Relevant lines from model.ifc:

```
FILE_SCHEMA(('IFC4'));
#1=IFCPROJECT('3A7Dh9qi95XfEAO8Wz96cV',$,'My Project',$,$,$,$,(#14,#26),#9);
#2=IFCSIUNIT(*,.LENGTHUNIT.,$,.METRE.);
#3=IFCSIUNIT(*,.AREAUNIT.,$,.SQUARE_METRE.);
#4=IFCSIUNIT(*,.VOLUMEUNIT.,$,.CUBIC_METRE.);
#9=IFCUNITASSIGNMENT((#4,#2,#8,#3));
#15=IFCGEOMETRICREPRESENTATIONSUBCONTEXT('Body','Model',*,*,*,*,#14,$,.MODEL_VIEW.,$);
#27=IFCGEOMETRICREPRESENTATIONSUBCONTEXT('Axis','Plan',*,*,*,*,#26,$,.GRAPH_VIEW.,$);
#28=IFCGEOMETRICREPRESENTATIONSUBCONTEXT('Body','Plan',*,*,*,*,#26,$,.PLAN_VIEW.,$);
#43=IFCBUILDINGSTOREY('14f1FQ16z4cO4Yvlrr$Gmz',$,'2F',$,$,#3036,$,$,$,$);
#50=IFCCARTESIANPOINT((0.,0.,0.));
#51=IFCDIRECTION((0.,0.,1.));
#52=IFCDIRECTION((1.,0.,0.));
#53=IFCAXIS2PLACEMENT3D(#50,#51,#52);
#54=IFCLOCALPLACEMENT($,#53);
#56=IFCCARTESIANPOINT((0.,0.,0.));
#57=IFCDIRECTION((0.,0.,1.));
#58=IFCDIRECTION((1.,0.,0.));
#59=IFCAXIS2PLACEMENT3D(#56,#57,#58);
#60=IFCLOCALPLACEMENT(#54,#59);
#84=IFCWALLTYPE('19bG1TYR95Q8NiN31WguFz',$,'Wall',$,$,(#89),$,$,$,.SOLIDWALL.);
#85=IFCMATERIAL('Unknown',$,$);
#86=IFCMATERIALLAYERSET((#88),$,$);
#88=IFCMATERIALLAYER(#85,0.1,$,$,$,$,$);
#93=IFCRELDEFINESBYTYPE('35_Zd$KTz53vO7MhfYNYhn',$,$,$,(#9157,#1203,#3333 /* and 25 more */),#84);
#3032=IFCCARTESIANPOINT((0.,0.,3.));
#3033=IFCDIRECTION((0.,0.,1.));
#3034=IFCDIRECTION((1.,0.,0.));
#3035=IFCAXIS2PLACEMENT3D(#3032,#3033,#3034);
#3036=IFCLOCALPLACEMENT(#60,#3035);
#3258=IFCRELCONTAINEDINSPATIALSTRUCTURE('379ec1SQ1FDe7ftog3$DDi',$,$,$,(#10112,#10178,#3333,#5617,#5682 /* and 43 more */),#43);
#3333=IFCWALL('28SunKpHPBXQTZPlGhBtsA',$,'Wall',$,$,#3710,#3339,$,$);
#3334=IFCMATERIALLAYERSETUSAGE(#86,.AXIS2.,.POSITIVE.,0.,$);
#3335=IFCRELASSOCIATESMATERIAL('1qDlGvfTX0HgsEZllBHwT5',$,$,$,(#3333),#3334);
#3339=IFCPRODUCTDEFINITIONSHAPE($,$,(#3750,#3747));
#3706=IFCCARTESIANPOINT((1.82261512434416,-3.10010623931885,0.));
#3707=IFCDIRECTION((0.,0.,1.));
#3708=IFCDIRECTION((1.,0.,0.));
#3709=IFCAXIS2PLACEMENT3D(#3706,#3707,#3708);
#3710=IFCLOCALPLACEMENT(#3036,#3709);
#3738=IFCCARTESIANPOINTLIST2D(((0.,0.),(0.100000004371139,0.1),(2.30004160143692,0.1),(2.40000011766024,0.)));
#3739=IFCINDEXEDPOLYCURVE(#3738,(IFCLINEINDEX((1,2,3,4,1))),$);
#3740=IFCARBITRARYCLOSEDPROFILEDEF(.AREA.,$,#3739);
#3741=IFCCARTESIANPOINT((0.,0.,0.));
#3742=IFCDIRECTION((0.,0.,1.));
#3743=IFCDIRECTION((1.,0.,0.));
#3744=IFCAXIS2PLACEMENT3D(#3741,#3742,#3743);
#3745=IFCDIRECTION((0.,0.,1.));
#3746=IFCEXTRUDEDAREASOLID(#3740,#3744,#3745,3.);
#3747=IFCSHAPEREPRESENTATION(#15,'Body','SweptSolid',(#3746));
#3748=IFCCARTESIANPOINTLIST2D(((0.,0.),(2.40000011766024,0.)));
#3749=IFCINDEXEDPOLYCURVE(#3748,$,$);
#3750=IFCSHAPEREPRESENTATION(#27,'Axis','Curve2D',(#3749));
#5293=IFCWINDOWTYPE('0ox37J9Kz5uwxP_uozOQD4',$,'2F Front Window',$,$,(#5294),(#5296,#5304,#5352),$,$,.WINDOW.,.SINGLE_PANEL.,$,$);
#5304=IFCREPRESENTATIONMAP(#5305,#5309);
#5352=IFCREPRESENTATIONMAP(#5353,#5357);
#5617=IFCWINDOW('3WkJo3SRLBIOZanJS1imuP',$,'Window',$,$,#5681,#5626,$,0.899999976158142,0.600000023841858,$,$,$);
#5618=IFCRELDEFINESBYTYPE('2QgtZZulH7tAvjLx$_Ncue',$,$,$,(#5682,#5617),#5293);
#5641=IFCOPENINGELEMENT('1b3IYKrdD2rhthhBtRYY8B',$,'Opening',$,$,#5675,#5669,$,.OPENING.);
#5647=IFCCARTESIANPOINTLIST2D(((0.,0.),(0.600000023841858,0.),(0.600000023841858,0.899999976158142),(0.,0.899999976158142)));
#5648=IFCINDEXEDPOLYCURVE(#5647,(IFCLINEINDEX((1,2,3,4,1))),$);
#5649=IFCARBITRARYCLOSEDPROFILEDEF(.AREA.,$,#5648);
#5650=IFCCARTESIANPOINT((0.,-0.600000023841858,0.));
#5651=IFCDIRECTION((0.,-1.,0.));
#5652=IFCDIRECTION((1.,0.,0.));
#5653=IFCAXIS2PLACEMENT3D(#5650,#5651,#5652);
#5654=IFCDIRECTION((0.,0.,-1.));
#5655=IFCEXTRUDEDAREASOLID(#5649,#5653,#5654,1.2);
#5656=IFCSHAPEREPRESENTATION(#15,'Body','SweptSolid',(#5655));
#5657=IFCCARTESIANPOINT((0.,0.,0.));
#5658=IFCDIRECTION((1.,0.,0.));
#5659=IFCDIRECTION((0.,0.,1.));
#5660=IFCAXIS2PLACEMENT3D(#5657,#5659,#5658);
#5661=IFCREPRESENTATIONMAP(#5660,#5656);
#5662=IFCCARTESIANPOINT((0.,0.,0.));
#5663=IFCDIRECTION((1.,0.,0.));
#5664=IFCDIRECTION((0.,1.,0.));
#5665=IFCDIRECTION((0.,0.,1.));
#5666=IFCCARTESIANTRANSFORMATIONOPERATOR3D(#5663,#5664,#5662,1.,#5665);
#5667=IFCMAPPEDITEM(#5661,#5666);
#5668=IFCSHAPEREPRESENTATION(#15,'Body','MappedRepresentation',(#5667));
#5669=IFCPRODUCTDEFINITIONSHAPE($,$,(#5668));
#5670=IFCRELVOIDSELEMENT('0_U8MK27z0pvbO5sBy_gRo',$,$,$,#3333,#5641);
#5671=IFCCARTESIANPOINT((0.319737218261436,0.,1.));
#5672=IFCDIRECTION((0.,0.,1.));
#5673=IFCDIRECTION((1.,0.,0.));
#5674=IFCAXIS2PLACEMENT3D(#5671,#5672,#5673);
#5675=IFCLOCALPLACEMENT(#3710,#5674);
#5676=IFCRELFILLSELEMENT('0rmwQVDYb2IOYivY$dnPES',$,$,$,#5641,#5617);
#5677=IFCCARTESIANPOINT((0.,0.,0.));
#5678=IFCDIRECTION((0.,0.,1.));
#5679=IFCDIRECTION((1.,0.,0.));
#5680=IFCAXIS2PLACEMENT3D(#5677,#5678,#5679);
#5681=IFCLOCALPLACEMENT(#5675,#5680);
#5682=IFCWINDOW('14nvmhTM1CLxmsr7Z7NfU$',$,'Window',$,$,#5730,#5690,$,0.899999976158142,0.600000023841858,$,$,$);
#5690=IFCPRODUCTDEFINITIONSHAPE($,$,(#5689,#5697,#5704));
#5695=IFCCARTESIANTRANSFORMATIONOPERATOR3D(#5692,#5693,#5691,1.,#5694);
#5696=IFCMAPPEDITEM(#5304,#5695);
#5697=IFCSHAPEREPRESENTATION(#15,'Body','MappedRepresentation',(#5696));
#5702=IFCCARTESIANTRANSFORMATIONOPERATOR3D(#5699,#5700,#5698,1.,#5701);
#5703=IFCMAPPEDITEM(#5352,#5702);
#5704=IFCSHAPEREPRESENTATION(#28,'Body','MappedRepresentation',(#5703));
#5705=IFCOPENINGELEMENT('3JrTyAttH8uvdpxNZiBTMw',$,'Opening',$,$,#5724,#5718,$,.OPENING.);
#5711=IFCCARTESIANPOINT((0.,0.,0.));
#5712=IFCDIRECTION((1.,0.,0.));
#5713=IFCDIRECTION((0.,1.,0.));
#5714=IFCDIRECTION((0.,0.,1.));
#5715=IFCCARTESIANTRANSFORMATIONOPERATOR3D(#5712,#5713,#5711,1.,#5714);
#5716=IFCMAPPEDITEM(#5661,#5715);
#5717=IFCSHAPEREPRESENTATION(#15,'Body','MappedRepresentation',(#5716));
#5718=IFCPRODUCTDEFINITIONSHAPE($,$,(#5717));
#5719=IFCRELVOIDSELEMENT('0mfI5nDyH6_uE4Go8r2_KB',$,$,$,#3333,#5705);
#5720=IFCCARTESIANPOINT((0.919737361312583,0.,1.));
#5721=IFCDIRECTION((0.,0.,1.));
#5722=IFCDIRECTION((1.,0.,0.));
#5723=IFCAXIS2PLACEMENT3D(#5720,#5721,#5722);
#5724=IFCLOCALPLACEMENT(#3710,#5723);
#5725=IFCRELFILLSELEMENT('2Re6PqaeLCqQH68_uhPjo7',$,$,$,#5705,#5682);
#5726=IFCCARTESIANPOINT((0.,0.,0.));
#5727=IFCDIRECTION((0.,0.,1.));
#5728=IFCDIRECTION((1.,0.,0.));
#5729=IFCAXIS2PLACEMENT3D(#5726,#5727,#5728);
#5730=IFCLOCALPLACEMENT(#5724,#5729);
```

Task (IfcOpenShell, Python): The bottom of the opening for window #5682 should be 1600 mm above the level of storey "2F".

```python
import numpy as np
import ifcopenshell
import ifcopenshell.api.geometry
import ifcopenshell.geom
import ifcopenshell.util.element
import ifcopenshell.util.placement
import ifcopenshell.util.shape
import ifcopenshell.util.unit

model = ifcopenshell.open("model.ifc")
unit_scale = ifcopenshell.util.unit.calculate_unit_scale(model)

window = model.by_guid("14nvmhTM1CLxmsr7Z7NfU$")
opening = window.FillsVoids[0].RelatingOpeningElement
storey = ifcopenshell.util.element.get_container(window, ifc_class="IfcBuildingStorey")
level = ifcopenshell.util.placement.get_local_placement(storey.ObjectPlacement)[2, 3]

# The opening's origin need not be at the sill, so measure its lowest point.
shape = ifcopenshell.geom.create_shape(ifcopenshell.geom.settings(), opening)
bottom = ifcopenshell.util.shape.get_shape_bottom_elevation(shape, shape.geometry) / unit_scale
dz = level + 1.6 / unit_scale - bottom

shift = np.array([0.0, 0.0, dz])
# The window is placed relative to its opening, so it follows when the opening moves.
matrix = ifcopenshell.util.placement.get_local_placement(opening.ObjectPlacement)
matrix[:3, 3] += shift
ifcopenshell.api.geometry.edit_object_placement(
    model, product=opening, matrix=matrix, is_si=False, should_transform_children=True
)

print(f"moved by {dz * unit_scale:+.3f} m")

model.write("model_v2.ifc")
```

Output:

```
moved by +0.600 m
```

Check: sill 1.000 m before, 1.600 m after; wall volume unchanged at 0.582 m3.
